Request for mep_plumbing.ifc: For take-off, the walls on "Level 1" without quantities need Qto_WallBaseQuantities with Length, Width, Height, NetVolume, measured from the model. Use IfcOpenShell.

First a look at what the model holds.

```python
import ifcopenshell
import ifcopenshell.util.element
import ifcopenshell.util.unit

model = ifcopenshell.open("mep_plumbing.ifc")
print(model.schema)
for unit_type in ("LENGTHUNIT", "AREAUNIT", "VOLUMEUNIT"):
    print(unit_type, ifcopenshell.util.unit.calculate_unit_scale(model, unit_type))
storey = next(s for s in model.by_type("IfcBuildingStorey") if s.Name == "Level 1")
walls = [e for e in ifcopenshell.util.element.get_decomposition(storey) if e.is_a("IfcWall")]
for e in sorted(walls, key=lambda e: e.id()):
    print(e.id(), e.is_a(), e.Name, list(ifcopenshell.util.element.get_psets(e, qtos_only=True)), sep=" | ")
```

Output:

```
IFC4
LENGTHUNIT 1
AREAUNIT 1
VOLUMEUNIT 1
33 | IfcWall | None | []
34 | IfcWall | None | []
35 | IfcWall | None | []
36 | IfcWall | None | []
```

```python
import ifcopenshell
import ifcopenshell.api.pset
import ifcopenshell.geom
import ifcopenshell.util.element
import ifcopenshell.util.shape
import ifcopenshell.util.unit

model = ifcopenshell.open("mep_plumbing.ifc")
unit_scale = ifcopenshell.util.unit.calculate_unit_scale(model)
volume_scale = ifcopenshell.util.unit.calculate_unit_scale(model, "VOLUMEUNIT")
settings = ifcopenshell.geom.settings()

storey = next(s for s in model.by_type("IfcBuildingStorey") if s.Name == "Level 1")
walls = [e for e in ifcopenshell.util.element.get_decomposition(storey) if e.is_a("IfcWall")]

for e in sorted(walls, key=lambda e: e.id()):
    if ifcopenshell.util.element.get_psets(e, qtos_only=True, should_inherit=False):
        continue
    # Geometry comes back in metres, in the element's own axes.
    shape = ifcopenshell.geom.create_shape(settings, e)
    values = {
        "Length": ifcopenshell.util.shape.get_x(shape.geometry) / unit_scale,
        "Width": ifcopenshell.util.shape.get_y(shape.geometry) / unit_scale,
        "Height": ifcopenshell.util.shape.get_z(shape.geometry) / unit_scale,
        "NetVolume": ifcopenshell.util.shape.get_volume(shape.geometry) / volume_scale,
    }
    qto = ifcopenshell.api.pset.add_qto(model, product=e, name="Qto_WallBaseQuantities")
    ifcopenshell.api.pset.edit_qto(model, qto=qto, properties=values)
    print(e.id(), {k: round(v, 3) for k, v in values.items()})

model.write("mep_plumbing_rev.ifc")
```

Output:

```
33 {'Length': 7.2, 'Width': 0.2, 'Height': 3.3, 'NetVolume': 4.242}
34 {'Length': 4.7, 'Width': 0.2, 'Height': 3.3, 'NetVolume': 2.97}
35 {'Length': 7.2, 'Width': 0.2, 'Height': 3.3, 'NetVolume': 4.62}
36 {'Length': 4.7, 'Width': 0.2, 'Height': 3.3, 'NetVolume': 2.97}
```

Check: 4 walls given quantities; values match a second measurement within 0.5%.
